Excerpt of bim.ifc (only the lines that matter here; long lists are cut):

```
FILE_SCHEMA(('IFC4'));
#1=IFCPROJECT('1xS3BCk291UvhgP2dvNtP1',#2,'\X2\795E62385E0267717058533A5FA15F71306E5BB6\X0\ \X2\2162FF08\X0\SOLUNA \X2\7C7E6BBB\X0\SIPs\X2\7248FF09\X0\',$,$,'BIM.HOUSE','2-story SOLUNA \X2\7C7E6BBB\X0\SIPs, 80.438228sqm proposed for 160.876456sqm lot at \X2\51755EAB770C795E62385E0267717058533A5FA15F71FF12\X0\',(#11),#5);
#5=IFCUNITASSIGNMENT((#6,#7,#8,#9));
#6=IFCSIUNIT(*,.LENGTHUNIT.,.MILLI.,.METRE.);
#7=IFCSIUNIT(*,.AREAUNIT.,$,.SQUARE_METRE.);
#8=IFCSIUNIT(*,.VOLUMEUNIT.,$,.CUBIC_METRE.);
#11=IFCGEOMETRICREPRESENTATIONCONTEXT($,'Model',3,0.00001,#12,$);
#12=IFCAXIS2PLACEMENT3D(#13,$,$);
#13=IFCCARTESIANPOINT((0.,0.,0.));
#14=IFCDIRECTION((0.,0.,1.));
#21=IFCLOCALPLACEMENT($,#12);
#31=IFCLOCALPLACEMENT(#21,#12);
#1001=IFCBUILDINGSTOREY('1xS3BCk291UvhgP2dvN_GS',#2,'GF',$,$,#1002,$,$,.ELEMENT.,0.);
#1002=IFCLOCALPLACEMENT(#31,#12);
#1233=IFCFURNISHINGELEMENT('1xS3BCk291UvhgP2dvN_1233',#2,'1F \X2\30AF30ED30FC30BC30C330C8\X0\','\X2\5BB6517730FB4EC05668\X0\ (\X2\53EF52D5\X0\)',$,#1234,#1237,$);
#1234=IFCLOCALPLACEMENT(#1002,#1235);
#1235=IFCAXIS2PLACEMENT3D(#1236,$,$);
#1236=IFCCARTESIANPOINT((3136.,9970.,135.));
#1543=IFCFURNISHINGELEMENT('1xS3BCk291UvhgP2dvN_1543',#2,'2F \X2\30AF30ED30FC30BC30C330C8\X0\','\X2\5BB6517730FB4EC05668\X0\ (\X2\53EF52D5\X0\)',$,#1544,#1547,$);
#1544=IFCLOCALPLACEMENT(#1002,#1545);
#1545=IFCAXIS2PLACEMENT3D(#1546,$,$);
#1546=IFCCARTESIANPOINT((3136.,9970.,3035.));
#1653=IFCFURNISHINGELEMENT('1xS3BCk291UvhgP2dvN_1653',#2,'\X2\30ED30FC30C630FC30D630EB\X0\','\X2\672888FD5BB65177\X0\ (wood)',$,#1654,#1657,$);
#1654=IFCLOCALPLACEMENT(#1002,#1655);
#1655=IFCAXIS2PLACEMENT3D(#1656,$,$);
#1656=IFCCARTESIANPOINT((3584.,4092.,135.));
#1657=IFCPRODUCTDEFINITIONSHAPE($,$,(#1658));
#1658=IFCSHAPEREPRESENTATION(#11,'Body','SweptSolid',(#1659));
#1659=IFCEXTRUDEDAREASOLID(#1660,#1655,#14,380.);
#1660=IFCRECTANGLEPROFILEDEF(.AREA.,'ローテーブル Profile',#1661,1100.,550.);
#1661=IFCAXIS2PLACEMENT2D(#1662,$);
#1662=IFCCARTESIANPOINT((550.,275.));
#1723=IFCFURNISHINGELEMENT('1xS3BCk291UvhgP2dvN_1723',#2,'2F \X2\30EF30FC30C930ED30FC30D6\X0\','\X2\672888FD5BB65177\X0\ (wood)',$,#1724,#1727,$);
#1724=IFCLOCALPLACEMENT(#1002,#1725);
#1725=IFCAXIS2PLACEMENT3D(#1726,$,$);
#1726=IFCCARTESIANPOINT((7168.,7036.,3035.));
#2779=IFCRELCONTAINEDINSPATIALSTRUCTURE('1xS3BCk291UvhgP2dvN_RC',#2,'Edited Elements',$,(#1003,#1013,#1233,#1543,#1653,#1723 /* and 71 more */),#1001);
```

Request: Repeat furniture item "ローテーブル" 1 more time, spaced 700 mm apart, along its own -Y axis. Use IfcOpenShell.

```python
import ifcopenshell
import ifcopenshell.api.geometry
import ifcopenshell.api.root
import ifcopenshell.util.element
import ifcopenshell.util.placement
import ifcopenshell.util.unit

model = ifcopenshell.open("bim.ifc")
unit_scale = ifcopenshell.util.unit.calculate_unit_scale(model)


def reuse_history(source, copy):
    """copy_class also copies each property set's owner history, people and application; keep the originals."""
    for rel in copy.IsDefinedBy:
        if rel.is_a("IfcRelDefinesByProperties") and (history := rel.RelatingPropertyDefinition.OwnerHistory):
            rel.RelatingPropertyDefinition.OwnerHistory = source.OwnerHistory
            ifcopenshell.util.element.remove_deep2(model, history)


source = model.by_guid("1xS3BCk291UvhgP2dvN_1653")
base = ifcopenshell.util.placement.get_local_placement(source.ObjectPlacement)
step = -base[:3, 1] * 0.7 / unit_scale

for i in range(1, 2):
    copy = ifcopenshell.api.root.copy_class(model, product=source)
    copy.Representation = ifcopenshell.util.element.copy_deep(
        model, source.Representation, exclude=["IfcGeometricRepresentationContext", "IfcRepresentationMap"]
    )
    reuse_history(source, copy)
    matrix = base.copy()
    matrix[:3, 3] += i * step
    print("added at", matrix[:3, 3].round(3) + 0.0)
    ifcopenshell.api.geometry.edit_object_placement(model, product=copy, matrix=matrix, is_si=False)

model.write("bim_rev.ifc")
```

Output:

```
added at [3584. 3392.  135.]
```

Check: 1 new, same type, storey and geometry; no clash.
